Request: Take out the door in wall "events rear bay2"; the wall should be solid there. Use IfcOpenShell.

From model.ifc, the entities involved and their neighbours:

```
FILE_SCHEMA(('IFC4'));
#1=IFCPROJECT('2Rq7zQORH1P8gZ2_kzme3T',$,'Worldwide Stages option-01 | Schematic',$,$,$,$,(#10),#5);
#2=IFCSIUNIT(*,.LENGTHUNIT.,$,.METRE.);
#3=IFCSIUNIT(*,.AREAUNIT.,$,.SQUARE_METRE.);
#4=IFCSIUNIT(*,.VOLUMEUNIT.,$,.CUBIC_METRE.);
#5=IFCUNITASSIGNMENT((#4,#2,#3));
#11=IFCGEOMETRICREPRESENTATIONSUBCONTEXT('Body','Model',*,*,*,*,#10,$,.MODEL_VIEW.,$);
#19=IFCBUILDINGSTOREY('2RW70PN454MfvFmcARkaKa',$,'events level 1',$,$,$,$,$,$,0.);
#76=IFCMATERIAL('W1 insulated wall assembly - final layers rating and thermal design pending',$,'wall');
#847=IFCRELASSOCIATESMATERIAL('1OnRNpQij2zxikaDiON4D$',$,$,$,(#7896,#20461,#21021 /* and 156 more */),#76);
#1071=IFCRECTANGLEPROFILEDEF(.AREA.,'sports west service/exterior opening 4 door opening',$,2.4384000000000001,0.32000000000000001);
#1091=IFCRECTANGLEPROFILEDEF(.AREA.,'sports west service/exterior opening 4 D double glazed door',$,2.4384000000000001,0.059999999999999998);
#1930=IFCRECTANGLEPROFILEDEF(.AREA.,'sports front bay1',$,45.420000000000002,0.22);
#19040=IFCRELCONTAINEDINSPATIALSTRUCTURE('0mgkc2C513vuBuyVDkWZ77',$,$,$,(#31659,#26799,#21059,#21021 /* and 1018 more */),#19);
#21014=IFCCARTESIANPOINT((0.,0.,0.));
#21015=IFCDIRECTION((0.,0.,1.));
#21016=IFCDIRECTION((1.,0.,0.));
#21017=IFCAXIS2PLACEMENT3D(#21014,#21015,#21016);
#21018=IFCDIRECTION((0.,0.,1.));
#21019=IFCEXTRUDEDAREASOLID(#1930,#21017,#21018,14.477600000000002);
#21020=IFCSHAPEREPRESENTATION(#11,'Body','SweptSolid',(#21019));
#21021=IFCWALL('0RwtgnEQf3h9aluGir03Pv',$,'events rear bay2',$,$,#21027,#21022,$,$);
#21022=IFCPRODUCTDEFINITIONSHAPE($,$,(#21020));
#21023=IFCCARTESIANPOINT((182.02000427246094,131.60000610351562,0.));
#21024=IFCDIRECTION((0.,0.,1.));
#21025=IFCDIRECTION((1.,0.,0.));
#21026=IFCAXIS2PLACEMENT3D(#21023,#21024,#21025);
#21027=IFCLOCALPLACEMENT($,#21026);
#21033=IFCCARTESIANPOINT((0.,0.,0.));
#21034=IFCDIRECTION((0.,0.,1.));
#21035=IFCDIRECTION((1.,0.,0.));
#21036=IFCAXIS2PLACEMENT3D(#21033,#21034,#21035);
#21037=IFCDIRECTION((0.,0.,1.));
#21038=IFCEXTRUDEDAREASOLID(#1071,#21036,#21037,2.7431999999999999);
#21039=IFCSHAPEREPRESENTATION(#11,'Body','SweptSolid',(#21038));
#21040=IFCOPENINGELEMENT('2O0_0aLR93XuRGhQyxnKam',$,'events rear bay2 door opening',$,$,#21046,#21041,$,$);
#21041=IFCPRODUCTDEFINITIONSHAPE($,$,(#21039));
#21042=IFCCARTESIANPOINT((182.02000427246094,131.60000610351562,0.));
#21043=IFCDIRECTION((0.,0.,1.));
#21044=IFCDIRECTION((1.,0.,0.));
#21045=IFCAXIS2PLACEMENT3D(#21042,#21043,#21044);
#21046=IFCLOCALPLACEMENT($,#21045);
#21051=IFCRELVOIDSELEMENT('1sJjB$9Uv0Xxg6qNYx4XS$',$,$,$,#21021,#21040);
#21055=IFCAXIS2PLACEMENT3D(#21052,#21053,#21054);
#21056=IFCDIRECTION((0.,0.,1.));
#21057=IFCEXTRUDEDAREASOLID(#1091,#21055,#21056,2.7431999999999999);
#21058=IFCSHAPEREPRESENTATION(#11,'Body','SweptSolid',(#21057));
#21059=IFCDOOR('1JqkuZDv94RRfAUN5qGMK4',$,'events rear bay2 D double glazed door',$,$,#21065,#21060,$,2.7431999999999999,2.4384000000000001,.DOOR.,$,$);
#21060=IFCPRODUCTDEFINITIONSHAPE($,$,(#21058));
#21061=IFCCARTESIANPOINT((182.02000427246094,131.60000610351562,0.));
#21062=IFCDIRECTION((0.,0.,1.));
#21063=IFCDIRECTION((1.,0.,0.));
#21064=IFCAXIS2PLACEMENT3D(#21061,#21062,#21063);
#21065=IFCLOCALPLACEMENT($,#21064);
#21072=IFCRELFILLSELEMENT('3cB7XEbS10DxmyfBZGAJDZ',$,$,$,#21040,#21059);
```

```python
import ifcopenshell
import ifcopenshell.api.feature
import ifcopenshell.api.root
import ifcopenshell.geom
import ifcopenshell.util.shape

model = ifcopenshell.open("model.ifc")
settings = ifcopenshell.geom.settings()


def volume(element):
    """Net volume in cubic metres, openings subtracted."""
    shape = ifcopenshell.geom.create_shape(settings, element)
    return ifcopenshell.util.shape.get_volume(shape.geometry)


door = model.by_guid("1JqkuZDv94RRfAUN5qGMK4")
opening = door.FillsVoids[0].RelatingOpeningElement
wall = opening.VoidsElements[0].RelatingBuildingElement
before = volume(wall)

ifcopenshell.api.root.remove_product(model, product=door)
ifcopenshell.api.feature.remove_feature(model, feature=opening)

after = volume(wall)

print(f"wall volume {before:.3f} -> {after:.3f} m3")

model.write("model-out.ifc")
```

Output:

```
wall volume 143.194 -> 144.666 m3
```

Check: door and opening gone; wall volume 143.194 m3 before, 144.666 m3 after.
